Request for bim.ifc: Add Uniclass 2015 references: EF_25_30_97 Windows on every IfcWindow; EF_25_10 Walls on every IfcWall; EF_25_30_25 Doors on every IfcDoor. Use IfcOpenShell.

First a look at what the model holds.

```python
import ifcopenshell

model = ifcopenshell.open("bim.ifc")
print(model.schema)
print("classifications:", [c.Name for c in model.by_type("IfcClassification")])
for ifc_class in ("IfcDoor", "IfcRoof", "IfcStair", "IfcWall", "IfcWindow"):
    print(ifc_class, len(model.by_type(ifc_class)))
```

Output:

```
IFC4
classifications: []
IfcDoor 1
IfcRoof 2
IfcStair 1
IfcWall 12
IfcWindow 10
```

```python
import ifcopenshell
import ifcopenshell.api.classification

model = ifcopenshell.open("bim.ifc")

system = ifcopenshell.api.classification.add_classification(model, classification="Uniclass 2015")

codes = {
    "IfcWindow": ("EF_25_30_97", "Windows"),
    "IfcWall": ("EF_25_10", "Walls"),
    "IfcDoor": ("EF_25_30_25", "Doors"),
}
for ifc_class, (code, name) in codes.items():
    products = model.by_type(ifc_class)
    ifcopenshell.api.classification.add_reference(
        model, products=products, classification=system, identification=code, name=name
    )
    print(code, len(products))

model.write("bim_updated.ifc")
```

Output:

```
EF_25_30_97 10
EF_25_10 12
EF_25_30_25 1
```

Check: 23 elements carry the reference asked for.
